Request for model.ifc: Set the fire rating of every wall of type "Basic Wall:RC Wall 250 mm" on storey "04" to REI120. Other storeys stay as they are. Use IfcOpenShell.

First a look at what the model holds.

```python
import ifcopenshell
import ifcopenshell.util.element

model = ifcopenshell.open("model.ifc")
print(model.schema)
storey = next(s for s in model.by_type("IfcBuildingStorey") if s.Name == "04")
walls = [e for e in ifcopenshell.util.element.get_decomposition(storey) if e.is_a("IfcWall")]
seen = {}
for e in walls:
    element_type = ifcopenshell.util.element.get_type(e)
    key = (element_type.Name if element_type != e and element_type else None, ifcopenshell.util.element.get_pset(e, "Pset_WallCommon", "FireRating"))
    seen[key] = seen.get(key, 0) + 1
for (name, value), count in sorted(seen.items(), key=str):
    print(count, "x", name, "|", value)
```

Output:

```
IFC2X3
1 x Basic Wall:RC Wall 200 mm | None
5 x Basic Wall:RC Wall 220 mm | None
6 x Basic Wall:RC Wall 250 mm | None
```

```python
import ifcopenshell
import ifcopenshell.api.pset
import ifcopenshell.util.element

model = ifcopenshell.open("model.ifc")

storey = next(s for s in model.by_type("IfcBuildingStorey") if s.Name == "04")
walls = [e for e in ifcopenshell.util.element.get_decomposition(storey) if e.is_a("IfcWall")]

count = 0
for e in walls:
    element_type = ifcopenshell.util.element.get_type(e)
    if element_type in (None, e) or element_type.Name != "Basic Wall:RC Wall 250 mm":
        continue
    # add_pset returns the element's existing set when there is one.
    pset = ifcopenshell.api.pset.add_pset(model, product=e, name="Pset_WallCommon")
    ifcopenshell.api.pset.edit_pset(model, pset=pset, properties={"FireRating": "REI120"})
    count += 1

print(count, "walls updated")

model.write("model_updated.ifc")
```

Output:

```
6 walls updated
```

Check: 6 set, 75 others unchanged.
